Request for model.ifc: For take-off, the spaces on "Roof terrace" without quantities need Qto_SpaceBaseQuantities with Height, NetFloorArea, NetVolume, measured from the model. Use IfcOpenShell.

First a look at what the model holds.

```python
import ifcopenshell
import ifcopenshell.util.element
import ifcopenshell.util.unit

model = ifcopenshell.open("model.ifc")
print(model.schema)
for unit_type in ("LENGTHUNIT", "AREAUNIT", "VOLUMEUNIT"):
    print(unit_type, ifcopenshell.util.unit.calculate_unit_scale(model, unit_type))
storey = next(s for s in model.by_type("IfcBuildingStorey") if s.Name == "Roof terrace")
spaces = [e for e in ifcopenshell.util.element.get_decomposition(storey) if e.is_a("IfcSpace")]
for e in sorted(spaces, key=lambda e: e.id()):
    print(e.id(), e.is_a(), e.Name, list(ifcopenshell.util.element.get_psets(e, qtos_only=True)), sep=" | ")
```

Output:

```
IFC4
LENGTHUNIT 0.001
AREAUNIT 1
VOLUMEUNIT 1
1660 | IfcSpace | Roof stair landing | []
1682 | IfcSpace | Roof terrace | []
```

```python
import ifcopenshell
import ifcopenshell.api.pset
import ifcopenshell.geom
import ifcopenshell.util.element
import ifcopenshell.util.shape
import ifcopenshell.util.unit

model = ifcopenshell.open("model.ifc")
unit_scale = ifcopenshell.util.unit.calculate_unit_scale(model)
area_scale = ifcopenshell.util.unit.calculate_unit_scale(model, "AREAUNIT")
volume_scale = ifcopenshell.util.unit.calculate_unit_scale(model, "VOLUMEUNIT")
settings = ifcopenshell.geom.settings()

storey = next(s for s in model.by_type("IfcBuildingStorey") if s.Name == "Roof terrace")
spaces = [e for e in ifcopenshell.util.element.get_decomposition(storey) if e.is_a("IfcSpace")]

for e in sorted(spaces, key=lambda e: e.id()):
    if ifcopenshell.util.element.get_psets(e, qtos_only=True, should_inherit=False):
        continue
    # Geometry comes back in metres, in the element's own axes.
    shape = ifcopenshell.geom.create_shape(settings, e)
    values = {
        "Height": ifcopenshell.util.shape.get_z(shape.geometry) / unit_scale,
        "NetFloorArea": ifcopenshell.util.shape.get_footprint_area(shape.geometry) / area_scale,
        "NetVolume": ifcopenshell.util.shape.get_volume(shape.geometry) / volume_scale,
    }
    qto = ifcopenshell.api.pset.add_qto(model, product=e, name="Qto_SpaceBaseQuantities")
    ifcopenshell.api.pset.edit_qto(model, qto=qto, properties=values)
    print(e.id(), {k: round(v, 3) for k, v in values.items()})

model.write("model_updated.ifc")
```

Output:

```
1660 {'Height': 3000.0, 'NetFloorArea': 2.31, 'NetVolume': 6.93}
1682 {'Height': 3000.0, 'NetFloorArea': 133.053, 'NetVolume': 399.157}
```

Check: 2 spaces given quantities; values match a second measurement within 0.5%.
